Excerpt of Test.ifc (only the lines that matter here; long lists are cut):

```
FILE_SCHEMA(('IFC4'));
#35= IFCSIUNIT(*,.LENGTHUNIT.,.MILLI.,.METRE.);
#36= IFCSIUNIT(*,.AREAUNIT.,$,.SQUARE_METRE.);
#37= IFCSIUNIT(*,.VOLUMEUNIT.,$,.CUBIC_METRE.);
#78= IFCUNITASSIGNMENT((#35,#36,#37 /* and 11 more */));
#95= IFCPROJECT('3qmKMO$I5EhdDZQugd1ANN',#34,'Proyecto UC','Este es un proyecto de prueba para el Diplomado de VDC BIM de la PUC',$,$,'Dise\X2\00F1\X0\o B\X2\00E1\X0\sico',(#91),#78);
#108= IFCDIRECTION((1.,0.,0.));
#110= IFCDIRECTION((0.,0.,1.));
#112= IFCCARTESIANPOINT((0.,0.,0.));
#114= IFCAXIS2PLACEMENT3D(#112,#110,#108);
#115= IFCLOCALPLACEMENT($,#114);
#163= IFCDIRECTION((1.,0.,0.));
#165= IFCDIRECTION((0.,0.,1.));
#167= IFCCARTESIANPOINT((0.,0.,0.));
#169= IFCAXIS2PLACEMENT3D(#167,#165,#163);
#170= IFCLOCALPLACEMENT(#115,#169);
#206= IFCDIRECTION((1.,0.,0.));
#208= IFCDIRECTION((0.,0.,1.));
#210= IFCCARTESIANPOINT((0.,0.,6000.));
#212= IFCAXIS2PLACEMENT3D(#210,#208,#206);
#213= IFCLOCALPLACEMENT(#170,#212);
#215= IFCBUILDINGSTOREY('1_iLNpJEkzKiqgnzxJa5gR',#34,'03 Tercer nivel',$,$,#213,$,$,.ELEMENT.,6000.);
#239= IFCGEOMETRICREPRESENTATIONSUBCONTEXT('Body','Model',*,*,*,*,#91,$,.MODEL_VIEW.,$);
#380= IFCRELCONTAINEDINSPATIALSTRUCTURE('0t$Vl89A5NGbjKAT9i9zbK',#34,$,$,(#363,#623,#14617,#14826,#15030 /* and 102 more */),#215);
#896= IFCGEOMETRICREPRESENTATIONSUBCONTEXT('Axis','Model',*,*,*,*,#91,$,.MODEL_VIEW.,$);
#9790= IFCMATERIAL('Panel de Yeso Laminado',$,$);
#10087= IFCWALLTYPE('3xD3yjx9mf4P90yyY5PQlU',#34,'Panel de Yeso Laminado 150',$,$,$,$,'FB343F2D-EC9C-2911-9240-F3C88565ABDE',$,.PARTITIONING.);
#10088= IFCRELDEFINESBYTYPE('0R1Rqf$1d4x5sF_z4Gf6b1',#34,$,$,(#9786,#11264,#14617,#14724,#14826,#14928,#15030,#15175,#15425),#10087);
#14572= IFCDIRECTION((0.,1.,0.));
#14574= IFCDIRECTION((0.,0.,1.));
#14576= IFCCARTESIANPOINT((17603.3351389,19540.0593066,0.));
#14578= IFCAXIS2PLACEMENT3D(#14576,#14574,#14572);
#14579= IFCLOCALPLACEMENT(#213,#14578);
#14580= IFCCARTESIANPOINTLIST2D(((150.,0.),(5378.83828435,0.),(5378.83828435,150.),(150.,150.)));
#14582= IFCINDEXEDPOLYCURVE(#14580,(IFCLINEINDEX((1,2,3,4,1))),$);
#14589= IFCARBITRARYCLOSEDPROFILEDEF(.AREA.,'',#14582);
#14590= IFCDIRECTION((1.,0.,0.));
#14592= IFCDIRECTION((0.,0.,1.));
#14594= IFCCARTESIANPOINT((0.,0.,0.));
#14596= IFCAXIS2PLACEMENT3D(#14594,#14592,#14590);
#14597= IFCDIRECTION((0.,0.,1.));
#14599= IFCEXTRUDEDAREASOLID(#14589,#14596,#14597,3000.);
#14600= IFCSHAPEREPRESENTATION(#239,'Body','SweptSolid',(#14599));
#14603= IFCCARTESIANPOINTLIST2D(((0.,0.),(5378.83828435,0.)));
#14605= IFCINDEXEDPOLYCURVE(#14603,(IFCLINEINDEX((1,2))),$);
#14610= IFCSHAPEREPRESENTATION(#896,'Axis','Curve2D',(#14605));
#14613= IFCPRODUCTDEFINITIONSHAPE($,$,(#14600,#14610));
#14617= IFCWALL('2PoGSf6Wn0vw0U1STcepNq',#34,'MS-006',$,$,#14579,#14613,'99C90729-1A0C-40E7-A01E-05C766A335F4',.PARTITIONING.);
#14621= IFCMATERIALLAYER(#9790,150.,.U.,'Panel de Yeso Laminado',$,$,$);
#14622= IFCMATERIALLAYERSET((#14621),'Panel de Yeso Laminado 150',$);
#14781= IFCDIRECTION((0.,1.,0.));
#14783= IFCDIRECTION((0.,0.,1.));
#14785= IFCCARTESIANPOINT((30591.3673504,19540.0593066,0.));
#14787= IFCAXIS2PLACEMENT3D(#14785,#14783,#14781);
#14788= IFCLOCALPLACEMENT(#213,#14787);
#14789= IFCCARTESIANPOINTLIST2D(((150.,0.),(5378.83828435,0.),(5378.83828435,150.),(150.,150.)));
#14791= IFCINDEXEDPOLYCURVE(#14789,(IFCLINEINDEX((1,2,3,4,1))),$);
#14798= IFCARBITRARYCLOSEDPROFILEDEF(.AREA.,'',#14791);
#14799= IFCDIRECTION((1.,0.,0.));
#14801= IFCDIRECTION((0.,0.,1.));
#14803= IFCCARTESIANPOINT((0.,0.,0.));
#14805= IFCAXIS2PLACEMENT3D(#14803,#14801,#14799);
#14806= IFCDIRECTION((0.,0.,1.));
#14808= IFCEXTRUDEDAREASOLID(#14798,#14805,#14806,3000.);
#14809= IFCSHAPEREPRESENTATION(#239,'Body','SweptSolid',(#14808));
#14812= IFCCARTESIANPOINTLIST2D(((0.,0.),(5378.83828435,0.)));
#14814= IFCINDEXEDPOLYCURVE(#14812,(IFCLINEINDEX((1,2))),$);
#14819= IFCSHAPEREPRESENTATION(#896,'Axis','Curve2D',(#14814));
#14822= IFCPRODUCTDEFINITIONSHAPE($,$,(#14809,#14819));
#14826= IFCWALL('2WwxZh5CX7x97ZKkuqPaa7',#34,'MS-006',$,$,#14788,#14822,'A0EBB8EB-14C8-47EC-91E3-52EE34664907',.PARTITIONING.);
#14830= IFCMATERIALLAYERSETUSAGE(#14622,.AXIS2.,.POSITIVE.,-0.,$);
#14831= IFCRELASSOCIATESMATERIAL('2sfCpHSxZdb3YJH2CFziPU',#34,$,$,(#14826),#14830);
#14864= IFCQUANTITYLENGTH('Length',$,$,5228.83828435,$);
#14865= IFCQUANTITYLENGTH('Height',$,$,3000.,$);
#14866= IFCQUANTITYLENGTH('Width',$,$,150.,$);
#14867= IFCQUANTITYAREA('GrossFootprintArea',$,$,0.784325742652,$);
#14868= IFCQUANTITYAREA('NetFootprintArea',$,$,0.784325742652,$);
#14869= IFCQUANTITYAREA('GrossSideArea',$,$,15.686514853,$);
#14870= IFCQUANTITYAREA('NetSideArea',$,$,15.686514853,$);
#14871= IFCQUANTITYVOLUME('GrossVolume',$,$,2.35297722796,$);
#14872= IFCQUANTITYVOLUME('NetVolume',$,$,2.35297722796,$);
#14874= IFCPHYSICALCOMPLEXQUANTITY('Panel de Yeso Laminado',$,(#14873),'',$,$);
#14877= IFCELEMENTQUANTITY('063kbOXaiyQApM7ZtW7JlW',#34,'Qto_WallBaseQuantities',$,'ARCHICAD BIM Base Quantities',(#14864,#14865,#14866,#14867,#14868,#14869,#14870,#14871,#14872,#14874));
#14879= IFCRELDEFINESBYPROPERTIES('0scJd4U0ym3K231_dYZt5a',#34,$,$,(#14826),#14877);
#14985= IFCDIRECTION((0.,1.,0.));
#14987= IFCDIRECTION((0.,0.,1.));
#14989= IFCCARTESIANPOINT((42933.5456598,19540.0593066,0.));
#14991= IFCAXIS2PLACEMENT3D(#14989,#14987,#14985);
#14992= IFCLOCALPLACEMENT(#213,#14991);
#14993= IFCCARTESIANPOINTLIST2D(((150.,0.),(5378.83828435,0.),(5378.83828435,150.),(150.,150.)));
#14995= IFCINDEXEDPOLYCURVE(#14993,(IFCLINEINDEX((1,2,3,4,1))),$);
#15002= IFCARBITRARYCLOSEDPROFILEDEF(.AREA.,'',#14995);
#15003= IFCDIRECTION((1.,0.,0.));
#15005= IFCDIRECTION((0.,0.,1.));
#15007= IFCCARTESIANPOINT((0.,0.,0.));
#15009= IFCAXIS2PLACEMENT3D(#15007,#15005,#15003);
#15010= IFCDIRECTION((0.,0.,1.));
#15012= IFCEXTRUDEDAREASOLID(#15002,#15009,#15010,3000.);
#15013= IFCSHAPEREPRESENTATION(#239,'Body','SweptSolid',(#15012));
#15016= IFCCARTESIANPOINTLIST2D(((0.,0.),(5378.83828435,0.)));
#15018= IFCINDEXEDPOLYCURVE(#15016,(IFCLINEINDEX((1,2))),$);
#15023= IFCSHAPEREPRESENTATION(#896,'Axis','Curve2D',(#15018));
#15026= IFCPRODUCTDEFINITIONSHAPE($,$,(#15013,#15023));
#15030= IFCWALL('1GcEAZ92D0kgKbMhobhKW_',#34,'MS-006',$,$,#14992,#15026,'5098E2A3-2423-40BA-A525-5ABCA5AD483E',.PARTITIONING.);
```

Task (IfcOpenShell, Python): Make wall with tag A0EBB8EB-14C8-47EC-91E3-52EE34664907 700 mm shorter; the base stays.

```python
import ifcopenshell
import ifcopenshell.api.pset
import ifcopenshell.geom
import ifcopenshell.util.element
import ifcopenshell.util.representation
import ifcopenshell.util.shape
import ifcopenshell.util.unit

model = ifcopenshell.open("Test.ifc")
unit_scale = ifcopenshell.util.unit.calculate_unit_scale(model)
area_scale = ifcopenshell.util.unit.calculate_unit_scale(model, "AREAUNIT")
volume_scale = ifcopenshell.util.unit.calculate_unit_scale(model, "VOLUMEUNIT")
settings = ifcopenshell.geom.settings()


def volume(element):
    """Net volume in cubic metres, openings subtracted."""
    shape = ifcopenshell.geom.create_shape(settings, element)
    return ifcopenshell.util.shape.get_volume(shape.geometry)


wall = model.by_guid("2WwxZh5CX7x97ZKkuqPaa7")
before = volume(wall)

body = ifcopenshell.util.representation.get_representation(wall, "Model", "Body")
solid = body.Items[0]
old_height = solid.Depth
solid.Depth -= 700.0
after = volume(wall)
thickness = 0.15  # wall thickness in metres

# Update the stored height, areas and volumes.
qto = model.by_id(ifcopenshell.util.element.get_pset(wall, "Qto_WallBaseQuantities", should_inherit=False)["id"])
ifcopenshell.api.pset.edit_qto(model, qto=qto, properties={
    "Height": solid.Depth,
    "GrossSideArea": ifcopenshell.util.element.get_pset(wall, "Qto_WallBaseQuantities", "GrossSideArea") * solid.Depth / old_height,
    "NetSideArea": after / thickness / area_scale,
    "GrossVolume": ifcopenshell.util.element.get_pset(wall, "Qto_WallBaseQuantities", "GrossVolume") * solid.Depth / old_height,
    "NetVolume": after / volume_scale,
})

print(f"height {old_height:g} -> {solid.Depth:g}, volume {before:.3f} -> {after:.3f} m3")

model.write("Test-out.ifc")
```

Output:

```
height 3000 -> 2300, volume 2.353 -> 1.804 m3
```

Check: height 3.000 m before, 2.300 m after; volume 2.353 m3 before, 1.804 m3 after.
